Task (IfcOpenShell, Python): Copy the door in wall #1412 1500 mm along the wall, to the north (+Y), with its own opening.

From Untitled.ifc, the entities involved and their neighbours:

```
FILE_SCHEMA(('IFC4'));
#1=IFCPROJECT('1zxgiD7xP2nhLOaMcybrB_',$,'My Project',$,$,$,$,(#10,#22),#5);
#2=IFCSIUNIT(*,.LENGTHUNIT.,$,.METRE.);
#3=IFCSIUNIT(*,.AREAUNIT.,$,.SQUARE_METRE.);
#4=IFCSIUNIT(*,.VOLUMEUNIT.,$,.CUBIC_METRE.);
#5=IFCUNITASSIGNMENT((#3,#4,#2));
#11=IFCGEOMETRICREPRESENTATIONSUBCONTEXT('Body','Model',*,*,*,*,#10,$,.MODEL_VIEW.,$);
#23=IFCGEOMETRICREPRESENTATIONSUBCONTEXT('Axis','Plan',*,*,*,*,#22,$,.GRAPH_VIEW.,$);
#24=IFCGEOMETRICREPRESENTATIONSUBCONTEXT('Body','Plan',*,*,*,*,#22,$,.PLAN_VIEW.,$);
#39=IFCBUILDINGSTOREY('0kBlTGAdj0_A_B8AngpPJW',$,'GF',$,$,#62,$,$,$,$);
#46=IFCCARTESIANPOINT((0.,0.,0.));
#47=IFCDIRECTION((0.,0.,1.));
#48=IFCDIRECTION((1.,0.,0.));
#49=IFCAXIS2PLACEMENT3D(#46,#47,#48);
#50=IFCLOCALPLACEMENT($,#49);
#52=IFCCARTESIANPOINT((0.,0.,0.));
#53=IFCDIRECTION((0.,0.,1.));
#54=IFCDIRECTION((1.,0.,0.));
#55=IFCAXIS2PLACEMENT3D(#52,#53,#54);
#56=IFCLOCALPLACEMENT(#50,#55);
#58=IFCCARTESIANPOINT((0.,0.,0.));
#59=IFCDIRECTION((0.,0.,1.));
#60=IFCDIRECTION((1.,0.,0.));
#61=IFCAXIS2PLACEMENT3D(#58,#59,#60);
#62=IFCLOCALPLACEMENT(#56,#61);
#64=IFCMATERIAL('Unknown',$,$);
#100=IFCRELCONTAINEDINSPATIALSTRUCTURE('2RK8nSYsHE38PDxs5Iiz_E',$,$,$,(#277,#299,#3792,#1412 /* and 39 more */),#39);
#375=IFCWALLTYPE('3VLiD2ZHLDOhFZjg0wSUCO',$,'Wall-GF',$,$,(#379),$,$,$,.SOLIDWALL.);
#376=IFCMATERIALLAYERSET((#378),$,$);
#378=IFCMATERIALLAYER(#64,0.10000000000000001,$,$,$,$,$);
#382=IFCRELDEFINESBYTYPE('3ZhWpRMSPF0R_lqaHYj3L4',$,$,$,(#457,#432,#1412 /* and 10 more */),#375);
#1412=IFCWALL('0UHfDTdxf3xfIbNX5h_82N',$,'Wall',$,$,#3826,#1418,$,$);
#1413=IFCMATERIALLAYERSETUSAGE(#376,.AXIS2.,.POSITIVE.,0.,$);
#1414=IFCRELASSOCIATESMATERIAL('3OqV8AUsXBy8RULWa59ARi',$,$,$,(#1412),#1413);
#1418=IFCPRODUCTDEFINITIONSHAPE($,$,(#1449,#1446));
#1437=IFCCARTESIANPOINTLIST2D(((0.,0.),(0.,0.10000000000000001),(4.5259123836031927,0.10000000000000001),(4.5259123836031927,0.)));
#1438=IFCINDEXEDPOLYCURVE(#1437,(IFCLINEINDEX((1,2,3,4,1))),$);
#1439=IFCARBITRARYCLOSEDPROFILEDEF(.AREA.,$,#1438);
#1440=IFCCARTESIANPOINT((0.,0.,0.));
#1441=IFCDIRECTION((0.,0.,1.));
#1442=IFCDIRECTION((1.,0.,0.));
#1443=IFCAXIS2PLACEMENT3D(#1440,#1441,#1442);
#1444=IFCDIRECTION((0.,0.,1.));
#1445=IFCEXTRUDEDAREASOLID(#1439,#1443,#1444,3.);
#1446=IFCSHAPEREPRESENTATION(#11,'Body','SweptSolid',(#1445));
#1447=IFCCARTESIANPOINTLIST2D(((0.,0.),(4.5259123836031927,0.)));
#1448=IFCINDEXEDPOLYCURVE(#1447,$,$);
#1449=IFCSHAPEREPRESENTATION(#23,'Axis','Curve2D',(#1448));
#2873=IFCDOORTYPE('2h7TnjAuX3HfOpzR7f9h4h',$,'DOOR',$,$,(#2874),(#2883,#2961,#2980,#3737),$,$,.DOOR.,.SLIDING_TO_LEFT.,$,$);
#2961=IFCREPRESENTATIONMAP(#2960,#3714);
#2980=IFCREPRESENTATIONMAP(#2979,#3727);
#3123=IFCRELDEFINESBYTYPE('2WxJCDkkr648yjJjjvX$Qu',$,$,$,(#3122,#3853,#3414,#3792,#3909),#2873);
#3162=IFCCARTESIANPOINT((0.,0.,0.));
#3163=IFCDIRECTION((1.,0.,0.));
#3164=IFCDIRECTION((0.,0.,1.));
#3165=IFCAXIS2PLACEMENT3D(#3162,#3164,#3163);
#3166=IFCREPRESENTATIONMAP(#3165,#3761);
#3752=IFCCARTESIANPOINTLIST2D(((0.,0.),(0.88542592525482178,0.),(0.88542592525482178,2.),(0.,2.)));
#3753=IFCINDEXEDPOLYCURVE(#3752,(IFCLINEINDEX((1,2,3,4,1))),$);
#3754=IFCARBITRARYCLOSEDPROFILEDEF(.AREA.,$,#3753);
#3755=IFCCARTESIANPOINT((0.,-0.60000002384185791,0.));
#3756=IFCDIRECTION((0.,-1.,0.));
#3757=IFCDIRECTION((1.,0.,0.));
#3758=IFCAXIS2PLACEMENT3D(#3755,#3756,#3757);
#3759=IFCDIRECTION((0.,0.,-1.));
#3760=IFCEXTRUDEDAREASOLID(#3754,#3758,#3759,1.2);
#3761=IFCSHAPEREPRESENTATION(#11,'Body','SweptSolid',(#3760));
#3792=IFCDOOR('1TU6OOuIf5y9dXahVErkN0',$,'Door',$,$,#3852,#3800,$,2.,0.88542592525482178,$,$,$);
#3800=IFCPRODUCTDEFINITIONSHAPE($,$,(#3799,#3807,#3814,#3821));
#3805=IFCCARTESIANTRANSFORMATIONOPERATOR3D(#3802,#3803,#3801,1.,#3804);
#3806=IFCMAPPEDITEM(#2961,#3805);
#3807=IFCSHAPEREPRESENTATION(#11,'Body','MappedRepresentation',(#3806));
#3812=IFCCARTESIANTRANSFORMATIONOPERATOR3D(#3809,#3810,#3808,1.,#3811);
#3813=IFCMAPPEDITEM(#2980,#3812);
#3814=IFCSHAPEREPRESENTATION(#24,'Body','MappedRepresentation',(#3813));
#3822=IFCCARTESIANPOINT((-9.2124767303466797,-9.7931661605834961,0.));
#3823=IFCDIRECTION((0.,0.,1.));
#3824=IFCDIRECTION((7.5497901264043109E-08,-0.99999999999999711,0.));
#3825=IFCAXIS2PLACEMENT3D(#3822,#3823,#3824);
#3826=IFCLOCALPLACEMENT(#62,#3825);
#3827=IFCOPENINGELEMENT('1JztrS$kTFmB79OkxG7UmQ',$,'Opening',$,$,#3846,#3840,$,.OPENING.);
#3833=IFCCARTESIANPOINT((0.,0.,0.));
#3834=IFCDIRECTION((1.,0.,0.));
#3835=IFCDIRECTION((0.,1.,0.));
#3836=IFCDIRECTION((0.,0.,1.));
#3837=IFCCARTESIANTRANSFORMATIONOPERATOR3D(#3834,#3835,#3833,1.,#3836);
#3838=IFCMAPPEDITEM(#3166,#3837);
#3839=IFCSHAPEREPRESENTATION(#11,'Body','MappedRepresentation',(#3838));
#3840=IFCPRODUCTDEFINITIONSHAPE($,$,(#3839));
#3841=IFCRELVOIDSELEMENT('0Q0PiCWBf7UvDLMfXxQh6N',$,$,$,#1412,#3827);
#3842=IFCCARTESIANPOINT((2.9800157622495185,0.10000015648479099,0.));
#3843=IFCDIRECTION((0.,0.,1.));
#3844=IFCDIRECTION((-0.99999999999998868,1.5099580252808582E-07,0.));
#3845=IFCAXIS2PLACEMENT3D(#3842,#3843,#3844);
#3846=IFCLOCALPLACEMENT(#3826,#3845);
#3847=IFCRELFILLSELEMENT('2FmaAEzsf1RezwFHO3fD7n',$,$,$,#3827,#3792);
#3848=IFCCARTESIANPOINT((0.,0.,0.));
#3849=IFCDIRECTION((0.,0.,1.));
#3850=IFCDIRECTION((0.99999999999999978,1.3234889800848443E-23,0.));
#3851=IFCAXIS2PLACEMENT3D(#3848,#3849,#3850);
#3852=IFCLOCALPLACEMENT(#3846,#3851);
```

```python
import ifcopenshell
import ifcopenshell.api.feature
import ifcopenshell.api.geometry
import ifcopenshell.api.root
import ifcopenshell.geom
import ifcopenshell.util.element
import ifcopenshell.util.placement
import ifcopenshell.util.shape
import ifcopenshell.util.unit

model = ifcopenshell.open("Untitled.ifc")
unit_scale = ifcopenshell.util.unit.calculate_unit_scale(model)
settings = ifcopenshell.geom.settings()


def volume(element):
    """Net volume in cubic metres, openings subtracted."""
    shape = ifcopenshell.geom.create_shape(settings, element)
    return ifcopenshell.util.shape.get_volume(shape.geometry)


door = model.by_guid("1TU6OOuIf5y9dXahVErkN0")
opening = door.FillsVoids[0].RelatingOpeningElement
wall = opening.VoidsElements[0].RelatingBuildingElement
before = volume(wall)
shift = ifcopenshell.util.placement.get_local_placement(wall.ObjectPlacement)[:3, 0] * -1.5 / unit_scale

# copy_class copies the void relationship, type, container and properties, but no geometry.
new_opening = ifcopenshell.api.root.copy_class(model, product=opening)
new_opening.Representation = ifcopenshell.util.element.copy_deep(
    model, opening.Representation, exclude=["IfcGeometricRepresentationContext", "IfcRepresentationMap"]
)
new_door = ifcopenshell.api.root.copy_class(model, product=door)
new_door.Representation = ifcopenshell.util.element.copy_deep(
    model, door.Representation, exclude=["IfcGeometricRepresentationContext", "IfcRepresentationMap"]
)
ifcopenshell.api.feature.add_filling(model, opening=new_opening, element=new_door)

for old, new in ((opening, new_opening), (door, new_door)):
    matrix = ifcopenshell.util.placement.get_local_placement(old.ObjectPlacement)
    matrix[:3, 3] += shift
    ifcopenshell.api.geometry.edit_object_placement(model, product=new, matrix=matrix, is_si=False)

after = volume(wall)

print(f"wall volume {before:.3f} -> {after:.3f} m3")

model.write("Untitled_v2.ifc")
```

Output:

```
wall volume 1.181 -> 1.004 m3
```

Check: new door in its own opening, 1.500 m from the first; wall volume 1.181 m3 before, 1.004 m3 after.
